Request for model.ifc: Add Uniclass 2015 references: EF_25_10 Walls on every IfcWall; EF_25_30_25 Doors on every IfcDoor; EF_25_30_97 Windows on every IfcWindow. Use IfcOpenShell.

First a look at what the model holds.

```python
import ifcopenshell

model = ifcopenshell.open("model.ifc")
print(model.schema)
print("classifications:", [c.Name for c in model.by_type("IfcClassification")])
for ifc_class in ("IfcDoor", "IfcRoof", "IfcStair", "IfcWall", "IfcWindow"):
    print(ifc_class, len(model.by_type(ifc_class)))
```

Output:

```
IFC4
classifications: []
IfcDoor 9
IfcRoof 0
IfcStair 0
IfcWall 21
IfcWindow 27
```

```python
import ifcopenshell
import ifcopenshell.api.classification

model = ifcopenshell.open("model.ifc")

system = ifcopenshell.api.classification.add_classification(model, classification="Uniclass 2015")

codes = {
    "IfcWall": ("EF_25_10", "Walls"),
    "IfcDoor": ("EF_25_30_25", "Doors"),
    "IfcWindow": ("EF_25_30_97", "Windows"),
}
for ifc_class, (code, name) in codes.items():
    products = model.by_type(ifc_class)
    ifcopenshell.api.classification.add_reference(
        model, products=products, classification=system, identification=code, name=name
    )
    print(code, len(products))

model.write("model_edited.ifc")
```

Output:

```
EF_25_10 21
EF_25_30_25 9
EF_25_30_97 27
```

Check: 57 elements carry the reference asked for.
